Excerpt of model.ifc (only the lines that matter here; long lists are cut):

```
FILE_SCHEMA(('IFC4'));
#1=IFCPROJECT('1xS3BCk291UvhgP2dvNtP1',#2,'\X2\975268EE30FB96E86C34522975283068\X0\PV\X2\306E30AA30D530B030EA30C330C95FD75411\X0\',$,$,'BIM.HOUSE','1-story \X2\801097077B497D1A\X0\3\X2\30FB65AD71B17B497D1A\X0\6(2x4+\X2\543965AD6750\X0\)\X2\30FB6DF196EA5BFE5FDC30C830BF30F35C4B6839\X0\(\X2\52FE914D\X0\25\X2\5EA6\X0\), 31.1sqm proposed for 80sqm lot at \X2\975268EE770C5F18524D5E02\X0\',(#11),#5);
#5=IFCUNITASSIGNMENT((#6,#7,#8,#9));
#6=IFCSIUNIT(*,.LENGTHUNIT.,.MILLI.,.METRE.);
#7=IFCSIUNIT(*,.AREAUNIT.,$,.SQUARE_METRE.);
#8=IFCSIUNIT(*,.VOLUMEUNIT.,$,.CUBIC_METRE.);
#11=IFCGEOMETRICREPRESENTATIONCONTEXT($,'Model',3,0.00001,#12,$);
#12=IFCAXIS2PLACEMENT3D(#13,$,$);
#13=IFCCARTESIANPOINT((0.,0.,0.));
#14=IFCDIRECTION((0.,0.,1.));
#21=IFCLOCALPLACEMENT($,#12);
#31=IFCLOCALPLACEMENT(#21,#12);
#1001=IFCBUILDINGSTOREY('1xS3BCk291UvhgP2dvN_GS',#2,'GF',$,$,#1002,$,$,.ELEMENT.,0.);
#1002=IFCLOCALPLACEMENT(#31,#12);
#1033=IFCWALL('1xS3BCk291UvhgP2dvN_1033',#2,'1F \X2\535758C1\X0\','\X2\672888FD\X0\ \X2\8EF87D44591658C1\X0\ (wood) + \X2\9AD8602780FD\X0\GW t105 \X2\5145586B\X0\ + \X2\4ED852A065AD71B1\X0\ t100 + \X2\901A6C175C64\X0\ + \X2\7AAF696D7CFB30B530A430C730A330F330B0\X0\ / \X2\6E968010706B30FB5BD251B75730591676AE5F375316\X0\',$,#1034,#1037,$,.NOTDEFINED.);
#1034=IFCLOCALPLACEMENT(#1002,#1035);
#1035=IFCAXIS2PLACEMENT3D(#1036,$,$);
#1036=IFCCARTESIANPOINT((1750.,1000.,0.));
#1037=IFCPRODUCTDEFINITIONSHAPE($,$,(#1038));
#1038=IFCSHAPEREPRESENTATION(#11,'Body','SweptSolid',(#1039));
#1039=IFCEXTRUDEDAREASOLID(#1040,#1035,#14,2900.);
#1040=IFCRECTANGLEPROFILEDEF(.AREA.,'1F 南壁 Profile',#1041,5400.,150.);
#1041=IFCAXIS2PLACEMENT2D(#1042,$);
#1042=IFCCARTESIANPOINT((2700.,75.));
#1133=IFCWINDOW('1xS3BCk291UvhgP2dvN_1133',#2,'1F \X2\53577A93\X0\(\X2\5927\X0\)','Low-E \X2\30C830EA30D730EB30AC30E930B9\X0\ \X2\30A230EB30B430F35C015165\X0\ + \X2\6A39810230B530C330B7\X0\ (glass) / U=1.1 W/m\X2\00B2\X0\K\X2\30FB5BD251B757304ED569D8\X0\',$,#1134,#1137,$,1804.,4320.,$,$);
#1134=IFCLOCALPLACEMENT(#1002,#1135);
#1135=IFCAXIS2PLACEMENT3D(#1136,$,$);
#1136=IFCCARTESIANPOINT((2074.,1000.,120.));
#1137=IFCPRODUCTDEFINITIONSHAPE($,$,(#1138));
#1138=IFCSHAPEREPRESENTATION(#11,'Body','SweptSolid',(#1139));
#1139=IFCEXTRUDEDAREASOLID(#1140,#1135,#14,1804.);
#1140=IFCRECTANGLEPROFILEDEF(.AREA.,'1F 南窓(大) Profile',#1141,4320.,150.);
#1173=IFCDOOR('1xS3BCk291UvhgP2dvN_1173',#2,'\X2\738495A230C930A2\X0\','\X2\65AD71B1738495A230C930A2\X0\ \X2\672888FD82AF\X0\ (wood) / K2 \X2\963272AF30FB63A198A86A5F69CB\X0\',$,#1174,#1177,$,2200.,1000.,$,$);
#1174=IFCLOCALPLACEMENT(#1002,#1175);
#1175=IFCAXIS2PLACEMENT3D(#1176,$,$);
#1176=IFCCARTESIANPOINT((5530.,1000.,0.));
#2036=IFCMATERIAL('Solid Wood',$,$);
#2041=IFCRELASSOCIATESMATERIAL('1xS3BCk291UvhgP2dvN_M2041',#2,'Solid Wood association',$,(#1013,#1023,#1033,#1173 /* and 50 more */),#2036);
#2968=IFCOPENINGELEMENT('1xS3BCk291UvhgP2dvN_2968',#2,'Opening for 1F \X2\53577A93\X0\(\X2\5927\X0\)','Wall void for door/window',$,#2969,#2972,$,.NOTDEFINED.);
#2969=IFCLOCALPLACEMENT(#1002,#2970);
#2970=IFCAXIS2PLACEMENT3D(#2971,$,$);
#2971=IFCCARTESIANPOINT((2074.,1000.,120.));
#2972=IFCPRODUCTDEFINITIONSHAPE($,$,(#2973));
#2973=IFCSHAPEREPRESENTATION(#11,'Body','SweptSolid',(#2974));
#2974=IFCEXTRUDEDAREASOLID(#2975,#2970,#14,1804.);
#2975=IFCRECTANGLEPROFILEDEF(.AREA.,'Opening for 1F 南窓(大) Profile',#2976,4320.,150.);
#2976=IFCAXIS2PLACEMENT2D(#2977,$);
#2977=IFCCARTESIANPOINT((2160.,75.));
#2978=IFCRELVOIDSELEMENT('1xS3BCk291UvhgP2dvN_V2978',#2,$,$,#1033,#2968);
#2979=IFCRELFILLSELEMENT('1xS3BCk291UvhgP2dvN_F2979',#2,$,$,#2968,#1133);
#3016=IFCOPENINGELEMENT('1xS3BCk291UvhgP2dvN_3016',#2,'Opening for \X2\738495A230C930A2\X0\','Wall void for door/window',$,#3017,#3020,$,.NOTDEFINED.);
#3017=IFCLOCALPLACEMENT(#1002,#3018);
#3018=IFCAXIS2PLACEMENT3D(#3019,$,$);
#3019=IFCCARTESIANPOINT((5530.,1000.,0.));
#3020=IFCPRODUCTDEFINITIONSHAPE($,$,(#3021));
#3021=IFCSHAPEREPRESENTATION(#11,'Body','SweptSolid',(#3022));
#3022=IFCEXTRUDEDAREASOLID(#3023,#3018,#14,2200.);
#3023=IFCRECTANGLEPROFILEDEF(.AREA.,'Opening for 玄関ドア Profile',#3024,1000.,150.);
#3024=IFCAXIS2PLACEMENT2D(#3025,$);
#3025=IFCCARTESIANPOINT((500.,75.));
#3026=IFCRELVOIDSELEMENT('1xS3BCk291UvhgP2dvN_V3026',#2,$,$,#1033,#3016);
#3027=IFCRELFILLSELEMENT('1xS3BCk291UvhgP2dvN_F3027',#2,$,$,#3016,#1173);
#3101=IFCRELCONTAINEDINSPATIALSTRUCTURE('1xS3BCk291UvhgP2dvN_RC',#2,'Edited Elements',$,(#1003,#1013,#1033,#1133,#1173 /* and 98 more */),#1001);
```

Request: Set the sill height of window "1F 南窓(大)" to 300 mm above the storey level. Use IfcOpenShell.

```python
import numpy as np
import ifcopenshell
import ifcopenshell.api.geometry
import ifcopenshell.geom
import ifcopenshell.util.element
import ifcopenshell.util.placement
import ifcopenshell.util.shape
import ifcopenshell.util.unit

model = ifcopenshell.open("model.ifc")
unit_scale = ifcopenshell.util.unit.calculate_unit_scale(model)

window = model.by_guid("1xS3BCk291UvhgP2dvN_1133")
opening = window.FillsVoids[0].RelatingOpeningElement
storey = ifcopenshell.util.element.get_container(window, ifc_class="IfcBuildingStorey")
level = ifcopenshell.util.placement.get_local_placement(storey.ObjectPlacement)[2, 3]

# The opening's origin need not be at the sill, so measure its lowest point.
shape = ifcopenshell.geom.create_shape(ifcopenshell.geom.settings(), opening)
bottom = ifcopenshell.util.shape.get_shape_bottom_elevation(shape, shape.geometry) / unit_scale
dz = level + 300.0 - bottom

shift = np.array([0.0, 0.0, dz])
# The window is not placed relative to its opening, so move both.
for product in (opening, window):
    matrix = ifcopenshell.util.placement.get_local_placement(product.ObjectPlacement)
    matrix[:3, 3] += shift
    ifcopenshell.api.geometry.edit_object_placement(model, product=product, matrix=matrix, is_si=False)

print(f"moved by {dz * unit_scale:+.3f} m")

model.write("model_updated.ifc")
```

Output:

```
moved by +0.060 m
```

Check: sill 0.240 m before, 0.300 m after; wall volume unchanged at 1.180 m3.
